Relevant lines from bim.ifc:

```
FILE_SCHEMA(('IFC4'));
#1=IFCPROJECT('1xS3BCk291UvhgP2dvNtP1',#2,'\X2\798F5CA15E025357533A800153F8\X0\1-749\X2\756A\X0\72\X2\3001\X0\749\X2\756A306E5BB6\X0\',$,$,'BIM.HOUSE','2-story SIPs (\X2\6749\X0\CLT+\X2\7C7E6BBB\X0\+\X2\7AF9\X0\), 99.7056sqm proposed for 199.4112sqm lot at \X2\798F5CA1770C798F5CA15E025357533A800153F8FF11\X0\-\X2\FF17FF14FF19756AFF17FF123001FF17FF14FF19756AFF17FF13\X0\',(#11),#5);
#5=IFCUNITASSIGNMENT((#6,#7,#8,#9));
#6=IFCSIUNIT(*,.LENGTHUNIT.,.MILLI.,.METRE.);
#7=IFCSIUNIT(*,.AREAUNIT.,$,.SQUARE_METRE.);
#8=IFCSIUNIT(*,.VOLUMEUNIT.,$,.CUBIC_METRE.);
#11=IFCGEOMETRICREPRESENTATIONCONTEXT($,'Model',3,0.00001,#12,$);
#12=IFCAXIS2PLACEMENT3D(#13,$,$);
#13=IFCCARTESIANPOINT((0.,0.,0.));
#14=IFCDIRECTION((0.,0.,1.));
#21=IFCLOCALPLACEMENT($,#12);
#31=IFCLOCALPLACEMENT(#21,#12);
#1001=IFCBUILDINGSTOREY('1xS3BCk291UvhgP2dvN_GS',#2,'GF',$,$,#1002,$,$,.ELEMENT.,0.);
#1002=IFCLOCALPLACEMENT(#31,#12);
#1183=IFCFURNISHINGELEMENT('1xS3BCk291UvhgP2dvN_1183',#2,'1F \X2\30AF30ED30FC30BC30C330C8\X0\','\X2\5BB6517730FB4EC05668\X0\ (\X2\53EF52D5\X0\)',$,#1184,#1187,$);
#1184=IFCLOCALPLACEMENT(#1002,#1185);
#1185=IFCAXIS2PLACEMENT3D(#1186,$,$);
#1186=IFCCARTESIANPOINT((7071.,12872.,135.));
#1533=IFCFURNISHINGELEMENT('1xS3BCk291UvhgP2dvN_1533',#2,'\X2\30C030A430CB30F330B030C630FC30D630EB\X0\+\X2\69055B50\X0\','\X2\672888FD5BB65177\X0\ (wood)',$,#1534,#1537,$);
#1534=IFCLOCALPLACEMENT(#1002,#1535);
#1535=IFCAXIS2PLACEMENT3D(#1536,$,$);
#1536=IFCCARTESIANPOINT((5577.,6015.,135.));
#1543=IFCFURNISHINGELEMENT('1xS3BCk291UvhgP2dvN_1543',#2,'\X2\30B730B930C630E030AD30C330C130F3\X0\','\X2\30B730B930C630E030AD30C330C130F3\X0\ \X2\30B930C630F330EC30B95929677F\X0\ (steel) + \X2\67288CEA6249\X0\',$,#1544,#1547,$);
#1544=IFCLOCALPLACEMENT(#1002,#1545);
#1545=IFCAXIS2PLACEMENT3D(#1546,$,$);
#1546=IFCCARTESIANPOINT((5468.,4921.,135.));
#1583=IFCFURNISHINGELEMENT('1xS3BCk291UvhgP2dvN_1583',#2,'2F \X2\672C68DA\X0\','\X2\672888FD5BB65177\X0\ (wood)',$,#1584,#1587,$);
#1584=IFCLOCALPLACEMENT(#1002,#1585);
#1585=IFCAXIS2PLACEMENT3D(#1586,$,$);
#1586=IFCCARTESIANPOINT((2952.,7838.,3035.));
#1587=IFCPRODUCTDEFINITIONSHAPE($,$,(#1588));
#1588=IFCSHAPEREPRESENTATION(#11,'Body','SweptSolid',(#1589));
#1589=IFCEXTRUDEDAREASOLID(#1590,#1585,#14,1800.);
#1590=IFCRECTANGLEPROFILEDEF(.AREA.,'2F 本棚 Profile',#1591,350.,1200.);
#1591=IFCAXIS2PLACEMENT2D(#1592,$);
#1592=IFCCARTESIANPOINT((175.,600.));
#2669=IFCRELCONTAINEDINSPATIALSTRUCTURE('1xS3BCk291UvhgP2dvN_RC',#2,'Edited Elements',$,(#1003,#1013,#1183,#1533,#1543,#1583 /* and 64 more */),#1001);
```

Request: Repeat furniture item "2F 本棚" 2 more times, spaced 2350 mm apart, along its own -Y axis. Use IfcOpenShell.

```python
import ifcopenshell
import ifcopenshell.api.geometry
import ifcopenshell.api.root
import ifcopenshell.util.element
import ifcopenshell.util.placement
import ifcopenshell.util.unit

model = ifcopenshell.open("bim.ifc")
unit_scale = ifcopenshell.util.unit.calculate_unit_scale(model)


def reuse_history(source, copy):
    """copy_class also copies each property set's owner history, people and application; keep the originals."""
    for rel in copy.IsDefinedBy:
        if rel.is_a("IfcRelDefinesByProperties") and (history := rel.RelatingPropertyDefinition.OwnerHistory):
            rel.RelatingPropertyDefinition.OwnerHistory = source.OwnerHistory
            ifcopenshell.util.element.remove_deep2(model, history)


source = model.by_guid("1xS3BCk291UvhgP2dvN_1583")
base = ifcopenshell.util.placement.get_local_placement(source.ObjectPlacement)
step = -base[:3, 1] * 2.35 / unit_scale

for i in range(1, 3):
    copy = ifcopenshell.api.root.copy_class(model, product=source)
    copy.Representation = ifcopenshell.util.element.copy_deep(
        model, source.Representation, exclude=["IfcGeometricRepresentationContext", "IfcRepresentationMap"]
    )
    reuse_history(source, copy)
    matrix = base.copy()
    matrix[:3, 3] += i * step
    print("added at", matrix[:3, 3].round(3) + 0.0)
    ifcopenshell.api.geometry.edit_object_placement(model, product=copy, matrix=matrix, is_si=False)

model.write("bim-out.ifc")
```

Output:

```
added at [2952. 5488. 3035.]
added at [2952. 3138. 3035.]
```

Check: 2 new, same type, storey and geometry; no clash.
